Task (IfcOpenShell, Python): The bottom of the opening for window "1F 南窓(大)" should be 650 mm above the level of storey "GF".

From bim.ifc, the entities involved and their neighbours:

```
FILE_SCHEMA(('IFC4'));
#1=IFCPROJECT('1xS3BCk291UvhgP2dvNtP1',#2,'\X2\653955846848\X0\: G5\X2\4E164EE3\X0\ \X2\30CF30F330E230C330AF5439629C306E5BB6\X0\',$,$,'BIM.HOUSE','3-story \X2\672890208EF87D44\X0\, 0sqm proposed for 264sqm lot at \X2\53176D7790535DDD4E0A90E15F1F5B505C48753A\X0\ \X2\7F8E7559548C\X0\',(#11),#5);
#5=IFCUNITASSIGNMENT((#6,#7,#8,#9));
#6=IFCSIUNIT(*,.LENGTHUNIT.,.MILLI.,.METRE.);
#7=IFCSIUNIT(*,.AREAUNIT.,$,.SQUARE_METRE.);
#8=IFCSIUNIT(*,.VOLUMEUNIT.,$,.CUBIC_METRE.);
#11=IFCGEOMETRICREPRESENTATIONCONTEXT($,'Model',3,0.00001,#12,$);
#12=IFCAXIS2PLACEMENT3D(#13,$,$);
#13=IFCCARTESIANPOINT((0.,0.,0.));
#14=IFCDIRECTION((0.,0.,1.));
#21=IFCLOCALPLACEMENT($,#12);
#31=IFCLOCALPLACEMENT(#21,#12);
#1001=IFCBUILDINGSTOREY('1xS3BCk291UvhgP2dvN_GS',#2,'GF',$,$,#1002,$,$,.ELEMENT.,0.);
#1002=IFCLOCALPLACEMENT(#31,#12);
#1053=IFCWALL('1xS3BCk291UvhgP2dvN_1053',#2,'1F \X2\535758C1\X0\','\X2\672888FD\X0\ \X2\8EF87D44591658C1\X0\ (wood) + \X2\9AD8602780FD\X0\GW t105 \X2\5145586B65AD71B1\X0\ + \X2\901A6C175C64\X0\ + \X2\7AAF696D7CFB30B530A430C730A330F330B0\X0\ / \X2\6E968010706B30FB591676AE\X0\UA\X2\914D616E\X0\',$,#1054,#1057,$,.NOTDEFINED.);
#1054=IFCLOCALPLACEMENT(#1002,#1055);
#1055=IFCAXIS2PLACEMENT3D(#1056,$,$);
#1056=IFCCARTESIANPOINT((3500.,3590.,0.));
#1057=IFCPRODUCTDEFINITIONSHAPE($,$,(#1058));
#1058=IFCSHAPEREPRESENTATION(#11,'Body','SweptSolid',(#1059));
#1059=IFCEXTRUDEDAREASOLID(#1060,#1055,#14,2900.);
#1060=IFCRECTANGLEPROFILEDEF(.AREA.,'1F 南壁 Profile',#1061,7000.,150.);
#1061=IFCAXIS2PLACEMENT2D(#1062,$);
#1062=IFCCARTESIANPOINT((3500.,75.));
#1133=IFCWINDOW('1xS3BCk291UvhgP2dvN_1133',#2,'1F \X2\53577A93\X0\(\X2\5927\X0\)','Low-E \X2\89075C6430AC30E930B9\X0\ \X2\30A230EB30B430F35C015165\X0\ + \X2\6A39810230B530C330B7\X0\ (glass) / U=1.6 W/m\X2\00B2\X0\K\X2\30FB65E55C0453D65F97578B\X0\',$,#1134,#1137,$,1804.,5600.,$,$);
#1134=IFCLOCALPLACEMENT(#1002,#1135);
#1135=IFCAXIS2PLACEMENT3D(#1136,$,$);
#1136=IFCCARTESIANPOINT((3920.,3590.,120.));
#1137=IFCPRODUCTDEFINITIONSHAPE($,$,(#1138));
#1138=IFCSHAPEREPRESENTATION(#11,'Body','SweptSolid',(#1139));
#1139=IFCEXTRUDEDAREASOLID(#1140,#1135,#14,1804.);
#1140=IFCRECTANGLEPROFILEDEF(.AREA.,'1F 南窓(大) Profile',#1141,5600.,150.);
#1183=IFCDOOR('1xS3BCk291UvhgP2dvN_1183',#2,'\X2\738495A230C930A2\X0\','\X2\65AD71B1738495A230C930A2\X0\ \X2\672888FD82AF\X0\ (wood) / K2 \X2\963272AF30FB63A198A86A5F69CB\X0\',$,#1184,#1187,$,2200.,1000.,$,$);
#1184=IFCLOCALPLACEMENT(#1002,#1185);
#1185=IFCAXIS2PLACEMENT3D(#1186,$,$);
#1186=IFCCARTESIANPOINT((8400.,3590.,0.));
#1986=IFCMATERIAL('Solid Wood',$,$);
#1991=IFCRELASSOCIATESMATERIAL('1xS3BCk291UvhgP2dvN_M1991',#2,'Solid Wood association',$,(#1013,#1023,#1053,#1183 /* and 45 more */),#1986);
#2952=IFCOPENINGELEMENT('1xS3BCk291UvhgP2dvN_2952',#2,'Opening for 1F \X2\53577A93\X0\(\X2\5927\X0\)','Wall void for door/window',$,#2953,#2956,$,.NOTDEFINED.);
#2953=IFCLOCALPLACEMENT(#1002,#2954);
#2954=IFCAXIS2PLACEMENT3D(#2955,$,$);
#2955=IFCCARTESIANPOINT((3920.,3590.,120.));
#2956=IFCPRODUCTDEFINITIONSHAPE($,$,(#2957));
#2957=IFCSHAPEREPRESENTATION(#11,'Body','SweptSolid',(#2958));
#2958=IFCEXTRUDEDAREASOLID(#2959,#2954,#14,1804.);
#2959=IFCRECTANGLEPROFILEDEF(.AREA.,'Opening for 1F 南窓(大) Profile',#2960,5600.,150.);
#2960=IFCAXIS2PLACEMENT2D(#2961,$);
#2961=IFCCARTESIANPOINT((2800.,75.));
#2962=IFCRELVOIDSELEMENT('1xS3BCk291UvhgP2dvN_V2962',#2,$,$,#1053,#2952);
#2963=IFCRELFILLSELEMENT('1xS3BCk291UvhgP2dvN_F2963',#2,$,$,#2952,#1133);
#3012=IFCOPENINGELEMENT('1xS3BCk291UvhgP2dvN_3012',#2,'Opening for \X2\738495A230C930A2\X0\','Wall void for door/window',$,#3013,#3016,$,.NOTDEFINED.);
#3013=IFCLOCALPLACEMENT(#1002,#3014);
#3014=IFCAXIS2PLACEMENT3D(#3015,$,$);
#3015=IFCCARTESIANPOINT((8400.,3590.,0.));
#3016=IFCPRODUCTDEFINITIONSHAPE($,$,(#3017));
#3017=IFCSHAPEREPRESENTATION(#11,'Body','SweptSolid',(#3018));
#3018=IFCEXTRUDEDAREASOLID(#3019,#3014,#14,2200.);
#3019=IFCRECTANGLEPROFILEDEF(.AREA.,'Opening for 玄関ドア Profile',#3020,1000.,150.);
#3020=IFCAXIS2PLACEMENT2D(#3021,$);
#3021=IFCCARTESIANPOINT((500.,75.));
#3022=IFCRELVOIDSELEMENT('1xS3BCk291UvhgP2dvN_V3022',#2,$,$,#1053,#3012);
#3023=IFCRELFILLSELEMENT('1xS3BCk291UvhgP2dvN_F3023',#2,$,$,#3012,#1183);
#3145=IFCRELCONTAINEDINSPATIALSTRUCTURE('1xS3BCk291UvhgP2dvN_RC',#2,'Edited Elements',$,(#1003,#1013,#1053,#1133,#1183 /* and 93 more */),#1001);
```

```python
import numpy as np
import ifcopenshell
import ifcopenshell.api.geometry
import ifcopenshell.geom
import ifcopenshell.util.element
import ifcopenshell.util.placement
import ifcopenshell.util.shape
import ifcopenshell.util.unit

model = ifcopenshell.open("bim.ifc")
unit_scale = ifcopenshell.util.unit.calculate_unit_scale(model)

window = model.by_guid("1xS3BCk291UvhgP2dvN_1133")
opening = window.FillsVoids[0].RelatingOpeningElement
storey = ifcopenshell.util.element.get_container(window, ifc_class="IfcBuildingStorey")
level = ifcopenshell.util.placement.get_local_placement(storey.ObjectPlacement)[2, 3]

# The opening's origin need not be at the sill, so measure its lowest point.
shape = ifcopenshell.geom.create_shape(ifcopenshell.geom.settings(), opening)
bottom = ifcopenshell.util.shape.get_shape_bottom_elevation(shape, shape.geometry) / unit_scale
dz = level + 650.0 - bottom

shift = np.array([0.0, 0.0, dz])
# The window is not placed relative to its opening, so move both.
for product in (opening, window):
    matrix = ifcopenshell.util.placement.get_local_placement(product.ObjectPlacement)
    matrix[:3, 3] += shift
    ifcopenshell.api.geometry.edit_object_placement(model, product=product, matrix=matrix, is_si=False)

print(f"moved by {dz * unit_scale:+.3f} m")

model.write("bim-out.ifc")
```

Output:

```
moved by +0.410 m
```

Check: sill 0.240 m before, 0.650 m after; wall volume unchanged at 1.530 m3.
